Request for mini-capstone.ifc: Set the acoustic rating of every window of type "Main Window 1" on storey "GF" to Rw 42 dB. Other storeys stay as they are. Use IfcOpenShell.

First a look at what the model holds.

```python
import ifcopenshell
import ifcopenshell.util.element

model = ifcopenshell.open("mini-capstone.ifc")
print(model.schema)
storey = next(s for s in model.by_type("IfcBuildingStorey") if s.Name == "GF")
windows = [e for e in ifcopenshell.util.element.get_decomposition(storey) if e.is_a("IfcWindow")]
seen = {}
for e in windows:
    element_type = ifcopenshell.util.element.get_type(e)
    key = (element_type.Name if element_type != e and element_type else None, ifcopenshell.util.element.get_pset(e, "Pset_WindowCommon", "AcousticRating"))
    seen[key] = seen.get(key, 0) + 1
for (name, value), count in sorted(seen.items(), key=str):
    print(count, "x", name, "|", value)
```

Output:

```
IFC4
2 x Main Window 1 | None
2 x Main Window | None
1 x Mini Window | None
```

```python
import ifcopenshell
import ifcopenshell.api.pset
import ifcopenshell.util.element

model = ifcopenshell.open("mini-capstone.ifc")

storey = next(s for s in model.by_type("IfcBuildingStorey") if s.Name == "GF")
windows = [e for e in ifcopenshell.util.element.get_decomposition(storey) if e.is_a("IfcWindow")]

count = 0
for e in windows:
    element_type = ifcopenshell.util.element.get_type(e)
    if element_type in (None, e) or element_type.Name != "Main Window 1":
        continue
    # add_pset returns the element's existing set when there is one.
    pset = ifcopenshell.api.pset.add_pset(model, product=e, name="Pset_WindowCommon")
    ifcopenshell.api.pset.edit_pset(model, pset=pset, properties={"AcousticRating": "Rw 42 dB"})
    count += 1

print(count, "windows updated")

model.write("mini-capstone_v2.ifc")
```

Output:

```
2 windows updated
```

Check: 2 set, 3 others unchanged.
